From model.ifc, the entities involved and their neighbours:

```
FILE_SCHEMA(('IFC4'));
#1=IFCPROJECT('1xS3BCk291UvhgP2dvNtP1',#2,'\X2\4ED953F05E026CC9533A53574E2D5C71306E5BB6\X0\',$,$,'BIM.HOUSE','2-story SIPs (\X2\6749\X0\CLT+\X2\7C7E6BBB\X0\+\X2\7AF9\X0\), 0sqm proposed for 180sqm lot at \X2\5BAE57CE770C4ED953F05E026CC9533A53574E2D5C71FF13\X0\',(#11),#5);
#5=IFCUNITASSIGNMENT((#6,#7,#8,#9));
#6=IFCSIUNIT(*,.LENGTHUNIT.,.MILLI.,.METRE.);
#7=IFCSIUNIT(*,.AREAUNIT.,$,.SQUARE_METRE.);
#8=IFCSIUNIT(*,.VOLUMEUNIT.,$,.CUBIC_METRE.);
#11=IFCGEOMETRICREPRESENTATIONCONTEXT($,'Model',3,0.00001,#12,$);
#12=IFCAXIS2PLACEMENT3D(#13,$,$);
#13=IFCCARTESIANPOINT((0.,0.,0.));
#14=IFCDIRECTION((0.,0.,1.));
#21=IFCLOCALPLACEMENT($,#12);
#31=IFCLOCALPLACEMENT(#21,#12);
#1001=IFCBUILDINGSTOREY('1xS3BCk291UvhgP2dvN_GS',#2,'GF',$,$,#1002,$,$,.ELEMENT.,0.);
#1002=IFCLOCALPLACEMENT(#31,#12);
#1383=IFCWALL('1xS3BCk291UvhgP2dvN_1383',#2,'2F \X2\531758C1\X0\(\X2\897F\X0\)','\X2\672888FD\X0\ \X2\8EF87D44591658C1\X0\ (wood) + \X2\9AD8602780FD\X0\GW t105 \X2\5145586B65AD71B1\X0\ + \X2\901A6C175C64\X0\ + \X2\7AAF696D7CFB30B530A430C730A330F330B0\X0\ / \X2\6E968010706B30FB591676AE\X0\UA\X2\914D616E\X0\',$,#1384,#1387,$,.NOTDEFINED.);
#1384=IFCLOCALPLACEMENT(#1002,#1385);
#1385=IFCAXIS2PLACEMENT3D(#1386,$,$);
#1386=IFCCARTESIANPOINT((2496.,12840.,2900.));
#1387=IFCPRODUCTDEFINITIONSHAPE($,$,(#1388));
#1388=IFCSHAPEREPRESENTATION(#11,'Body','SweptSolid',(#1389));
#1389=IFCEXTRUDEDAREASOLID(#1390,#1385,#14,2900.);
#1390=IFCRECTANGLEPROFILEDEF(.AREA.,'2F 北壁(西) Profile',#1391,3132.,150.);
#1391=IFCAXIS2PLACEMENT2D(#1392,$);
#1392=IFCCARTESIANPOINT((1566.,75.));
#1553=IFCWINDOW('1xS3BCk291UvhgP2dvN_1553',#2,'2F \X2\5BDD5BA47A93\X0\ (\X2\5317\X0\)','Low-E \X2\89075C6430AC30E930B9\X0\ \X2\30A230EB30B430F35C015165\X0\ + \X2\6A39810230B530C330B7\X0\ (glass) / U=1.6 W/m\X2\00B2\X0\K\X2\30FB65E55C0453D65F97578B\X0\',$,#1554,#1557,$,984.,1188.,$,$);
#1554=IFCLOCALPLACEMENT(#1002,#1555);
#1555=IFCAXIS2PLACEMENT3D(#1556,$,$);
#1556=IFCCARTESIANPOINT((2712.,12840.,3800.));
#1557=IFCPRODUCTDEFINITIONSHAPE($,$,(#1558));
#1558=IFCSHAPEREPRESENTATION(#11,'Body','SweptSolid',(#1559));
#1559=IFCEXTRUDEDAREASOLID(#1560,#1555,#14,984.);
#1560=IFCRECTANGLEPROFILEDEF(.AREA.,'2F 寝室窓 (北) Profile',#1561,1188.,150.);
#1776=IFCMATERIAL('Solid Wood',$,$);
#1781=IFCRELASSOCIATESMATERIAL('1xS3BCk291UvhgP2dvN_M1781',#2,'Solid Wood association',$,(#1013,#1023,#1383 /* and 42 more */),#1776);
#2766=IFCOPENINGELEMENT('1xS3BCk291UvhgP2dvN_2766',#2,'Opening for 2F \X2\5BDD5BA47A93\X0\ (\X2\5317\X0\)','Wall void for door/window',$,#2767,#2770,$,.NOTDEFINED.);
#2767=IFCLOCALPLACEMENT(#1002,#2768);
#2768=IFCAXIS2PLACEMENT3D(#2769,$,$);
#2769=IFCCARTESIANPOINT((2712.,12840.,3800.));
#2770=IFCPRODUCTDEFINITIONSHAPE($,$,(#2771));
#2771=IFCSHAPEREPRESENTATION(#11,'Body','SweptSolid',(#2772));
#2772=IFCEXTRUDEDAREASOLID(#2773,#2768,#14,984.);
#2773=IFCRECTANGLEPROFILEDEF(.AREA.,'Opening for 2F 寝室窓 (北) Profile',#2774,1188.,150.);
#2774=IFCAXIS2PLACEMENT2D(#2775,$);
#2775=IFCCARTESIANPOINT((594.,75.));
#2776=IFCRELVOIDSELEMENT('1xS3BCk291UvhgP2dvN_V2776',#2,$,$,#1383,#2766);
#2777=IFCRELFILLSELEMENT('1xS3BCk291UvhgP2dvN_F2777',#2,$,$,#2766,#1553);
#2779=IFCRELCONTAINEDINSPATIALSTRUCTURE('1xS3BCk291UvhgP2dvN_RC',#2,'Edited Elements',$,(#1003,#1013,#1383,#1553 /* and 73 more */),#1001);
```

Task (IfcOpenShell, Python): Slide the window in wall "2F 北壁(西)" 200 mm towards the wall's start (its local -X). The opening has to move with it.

```python
import ifcopenshell
import ifcopenshell.api.geometry
import ifcopenshell.util.placement

model = ifcopenshell.open("model.ifc")

window = model.by_id(1553)
opening = window.FillsVoids[0].RelatingOpeningElement
wall = opening.VoidsElements[0].RelatingBuildingElement

wall_matrix = ifcopenshell.util.placement.get_local_placement(wall.ObjectPlacement)
shift = wall_matrix[:3, 0] * -200.0
before = ifcopenshell.util.placement.get_local_placement(window.ObjectPlacement)[:3, 3].copy()

# The window is not placed relative to its opening, so move both.
for product in (opening, window):
    matrix = ifcopenshell.util.placement.get_local_placement(product.ObjectPlacement)
    matrix[:3, 3] += shift
    ifcopenshell.api.geometry.edit_object_placement(model, product=product, matrix=matrix, is_si=False)

after = ifcopenshell.util.placement.get_local_placement(window.ObjectPlacement)[:3, 3]
print("window moved by", (after - before).round(3) + 0.0)

model.write("model_updated.ifc")
```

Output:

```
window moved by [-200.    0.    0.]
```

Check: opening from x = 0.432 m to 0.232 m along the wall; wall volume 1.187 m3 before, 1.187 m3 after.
